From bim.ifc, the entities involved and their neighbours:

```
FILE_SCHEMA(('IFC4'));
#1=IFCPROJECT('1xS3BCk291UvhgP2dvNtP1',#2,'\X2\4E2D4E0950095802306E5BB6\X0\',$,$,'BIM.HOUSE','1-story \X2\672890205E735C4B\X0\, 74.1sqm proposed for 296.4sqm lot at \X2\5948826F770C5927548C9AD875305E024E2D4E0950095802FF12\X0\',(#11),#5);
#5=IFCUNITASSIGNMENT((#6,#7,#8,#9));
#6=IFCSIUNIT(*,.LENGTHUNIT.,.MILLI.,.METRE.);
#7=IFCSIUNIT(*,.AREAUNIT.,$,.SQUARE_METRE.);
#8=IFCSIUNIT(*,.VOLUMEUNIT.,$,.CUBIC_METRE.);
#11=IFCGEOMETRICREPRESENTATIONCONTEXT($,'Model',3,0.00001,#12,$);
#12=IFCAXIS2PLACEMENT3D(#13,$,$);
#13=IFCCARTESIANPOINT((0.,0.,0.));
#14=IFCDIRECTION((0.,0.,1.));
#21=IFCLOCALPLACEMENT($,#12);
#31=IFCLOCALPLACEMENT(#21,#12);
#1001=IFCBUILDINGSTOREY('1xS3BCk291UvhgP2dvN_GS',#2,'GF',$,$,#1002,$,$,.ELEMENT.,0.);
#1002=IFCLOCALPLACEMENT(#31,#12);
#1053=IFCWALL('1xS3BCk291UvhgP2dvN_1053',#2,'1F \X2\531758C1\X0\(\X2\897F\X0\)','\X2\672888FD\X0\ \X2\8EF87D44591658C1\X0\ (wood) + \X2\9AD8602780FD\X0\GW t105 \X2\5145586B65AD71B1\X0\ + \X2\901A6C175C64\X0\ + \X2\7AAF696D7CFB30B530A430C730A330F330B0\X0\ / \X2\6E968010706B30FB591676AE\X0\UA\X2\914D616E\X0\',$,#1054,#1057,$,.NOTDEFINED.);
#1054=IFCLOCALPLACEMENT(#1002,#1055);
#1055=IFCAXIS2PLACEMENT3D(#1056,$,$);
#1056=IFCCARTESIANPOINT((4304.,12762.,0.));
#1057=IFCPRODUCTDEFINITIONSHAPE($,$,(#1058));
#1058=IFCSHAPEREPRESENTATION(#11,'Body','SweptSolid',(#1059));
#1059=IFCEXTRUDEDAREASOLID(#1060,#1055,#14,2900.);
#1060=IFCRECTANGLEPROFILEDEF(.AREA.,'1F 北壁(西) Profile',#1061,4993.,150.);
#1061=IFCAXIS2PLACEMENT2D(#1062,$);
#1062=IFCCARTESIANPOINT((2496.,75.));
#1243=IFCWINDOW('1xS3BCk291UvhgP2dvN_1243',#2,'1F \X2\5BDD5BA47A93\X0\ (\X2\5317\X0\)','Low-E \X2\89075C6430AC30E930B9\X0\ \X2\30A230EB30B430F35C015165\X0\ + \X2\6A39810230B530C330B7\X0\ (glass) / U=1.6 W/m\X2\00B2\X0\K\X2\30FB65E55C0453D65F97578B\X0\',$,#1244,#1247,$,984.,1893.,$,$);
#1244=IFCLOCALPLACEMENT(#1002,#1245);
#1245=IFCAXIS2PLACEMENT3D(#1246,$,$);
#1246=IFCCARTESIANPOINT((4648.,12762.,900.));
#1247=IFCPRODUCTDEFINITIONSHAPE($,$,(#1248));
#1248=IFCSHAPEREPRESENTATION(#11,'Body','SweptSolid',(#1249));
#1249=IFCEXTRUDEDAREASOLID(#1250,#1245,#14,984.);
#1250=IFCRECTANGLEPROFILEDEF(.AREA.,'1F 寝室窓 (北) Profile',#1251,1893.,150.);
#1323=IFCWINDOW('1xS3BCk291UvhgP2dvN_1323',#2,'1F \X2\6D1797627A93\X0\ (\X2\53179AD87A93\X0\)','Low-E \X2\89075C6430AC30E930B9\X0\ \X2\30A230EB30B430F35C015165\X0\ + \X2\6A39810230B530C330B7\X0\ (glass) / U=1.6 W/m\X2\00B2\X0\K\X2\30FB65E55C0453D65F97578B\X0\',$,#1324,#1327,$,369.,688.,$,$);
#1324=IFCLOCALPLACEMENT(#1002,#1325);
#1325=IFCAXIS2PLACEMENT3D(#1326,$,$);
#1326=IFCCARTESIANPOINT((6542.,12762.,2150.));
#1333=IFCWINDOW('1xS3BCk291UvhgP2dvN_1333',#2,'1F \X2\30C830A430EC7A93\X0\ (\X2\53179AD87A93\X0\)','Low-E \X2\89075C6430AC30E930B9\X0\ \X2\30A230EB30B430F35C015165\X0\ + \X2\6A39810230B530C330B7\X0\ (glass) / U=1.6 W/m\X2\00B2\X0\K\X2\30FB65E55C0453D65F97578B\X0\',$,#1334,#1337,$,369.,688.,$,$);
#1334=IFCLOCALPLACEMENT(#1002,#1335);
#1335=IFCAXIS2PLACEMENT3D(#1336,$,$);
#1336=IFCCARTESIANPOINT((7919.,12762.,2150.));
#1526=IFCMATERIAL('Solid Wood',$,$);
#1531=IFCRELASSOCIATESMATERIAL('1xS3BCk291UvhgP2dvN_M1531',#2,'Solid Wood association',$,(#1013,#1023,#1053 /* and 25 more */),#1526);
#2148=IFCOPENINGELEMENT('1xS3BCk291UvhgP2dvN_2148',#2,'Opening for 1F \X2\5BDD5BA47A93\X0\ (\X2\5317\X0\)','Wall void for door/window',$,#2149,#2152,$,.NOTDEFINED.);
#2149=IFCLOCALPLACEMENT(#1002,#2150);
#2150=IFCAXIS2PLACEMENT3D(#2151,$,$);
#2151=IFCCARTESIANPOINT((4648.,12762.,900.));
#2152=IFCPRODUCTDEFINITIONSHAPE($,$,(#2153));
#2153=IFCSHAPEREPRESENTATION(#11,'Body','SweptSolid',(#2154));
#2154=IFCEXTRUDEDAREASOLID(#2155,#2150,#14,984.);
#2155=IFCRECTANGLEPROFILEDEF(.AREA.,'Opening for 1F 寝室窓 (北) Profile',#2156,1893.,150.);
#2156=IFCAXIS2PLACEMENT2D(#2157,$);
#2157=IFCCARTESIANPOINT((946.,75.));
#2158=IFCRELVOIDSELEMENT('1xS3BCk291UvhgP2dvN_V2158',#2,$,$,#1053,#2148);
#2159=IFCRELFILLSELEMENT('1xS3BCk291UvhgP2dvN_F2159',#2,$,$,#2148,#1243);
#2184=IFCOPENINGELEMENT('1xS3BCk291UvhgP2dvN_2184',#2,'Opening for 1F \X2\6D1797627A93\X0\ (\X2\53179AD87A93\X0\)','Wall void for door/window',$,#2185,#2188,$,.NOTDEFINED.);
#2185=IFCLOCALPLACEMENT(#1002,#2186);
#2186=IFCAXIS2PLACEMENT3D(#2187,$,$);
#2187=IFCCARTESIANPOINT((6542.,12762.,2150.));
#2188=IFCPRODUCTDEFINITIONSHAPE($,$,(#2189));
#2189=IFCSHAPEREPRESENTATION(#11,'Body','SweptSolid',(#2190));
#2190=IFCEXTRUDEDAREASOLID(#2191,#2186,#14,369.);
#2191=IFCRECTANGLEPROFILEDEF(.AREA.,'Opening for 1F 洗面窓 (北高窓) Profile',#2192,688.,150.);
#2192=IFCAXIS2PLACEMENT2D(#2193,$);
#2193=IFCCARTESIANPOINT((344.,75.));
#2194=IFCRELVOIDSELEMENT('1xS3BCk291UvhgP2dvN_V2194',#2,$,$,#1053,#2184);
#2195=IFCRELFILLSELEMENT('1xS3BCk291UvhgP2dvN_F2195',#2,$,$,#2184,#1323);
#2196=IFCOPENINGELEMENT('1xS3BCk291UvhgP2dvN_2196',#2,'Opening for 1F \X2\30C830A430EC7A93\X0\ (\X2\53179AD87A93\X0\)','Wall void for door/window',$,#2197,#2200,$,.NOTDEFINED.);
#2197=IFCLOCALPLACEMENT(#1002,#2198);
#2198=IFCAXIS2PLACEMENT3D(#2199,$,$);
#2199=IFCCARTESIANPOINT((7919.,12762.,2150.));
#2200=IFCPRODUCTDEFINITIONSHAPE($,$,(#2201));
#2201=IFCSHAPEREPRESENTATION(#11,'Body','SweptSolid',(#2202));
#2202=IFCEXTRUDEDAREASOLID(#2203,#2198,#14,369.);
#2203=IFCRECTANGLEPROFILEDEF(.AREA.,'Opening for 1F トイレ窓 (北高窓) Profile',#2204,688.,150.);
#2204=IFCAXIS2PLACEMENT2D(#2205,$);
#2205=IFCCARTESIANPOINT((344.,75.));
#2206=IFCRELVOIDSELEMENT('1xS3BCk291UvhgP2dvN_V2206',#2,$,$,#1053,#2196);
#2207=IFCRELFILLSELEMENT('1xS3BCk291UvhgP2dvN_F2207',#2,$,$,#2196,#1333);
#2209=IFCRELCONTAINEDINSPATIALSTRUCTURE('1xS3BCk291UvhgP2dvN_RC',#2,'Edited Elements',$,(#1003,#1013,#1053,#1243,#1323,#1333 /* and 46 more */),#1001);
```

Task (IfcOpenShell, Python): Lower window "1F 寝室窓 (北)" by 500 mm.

```python
import numpy as np
import ifcopenshell
import ifcopenshell.api.geometry
import ifcopenshell.util.placement
import ifcopenshell.util.unit

model = ifcopenshell.open("bim.ifc")
unit_scale = ifcopenshell.util.unit.calculate_unit_scale(model)

window = model.by_guid("1xS3BCk291UvhgP2dvN_1243")
opening = window.FillsVoids[0].RelatingOpeningElement
dz = -0.5 / unit_scale

shift = np.array([0.0, 0.0, dz])
# The window is not placed relative to its opening, so move both.
for product in (opening, window):
    matrix = ifcopenshell.util.placement.get_local_placement(product.ObjectPlacement)
    matrix[:3, 3] += shift
    ifcopenshell.api.geometry.edit_object_placement(model, product=product, matrix=matrix, is_si=False)

print(f"moved by {dz * unit_scale:+.3f} m")

model.write("bim_edited.ifc")
```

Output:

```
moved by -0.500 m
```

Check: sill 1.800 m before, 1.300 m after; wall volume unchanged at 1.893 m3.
